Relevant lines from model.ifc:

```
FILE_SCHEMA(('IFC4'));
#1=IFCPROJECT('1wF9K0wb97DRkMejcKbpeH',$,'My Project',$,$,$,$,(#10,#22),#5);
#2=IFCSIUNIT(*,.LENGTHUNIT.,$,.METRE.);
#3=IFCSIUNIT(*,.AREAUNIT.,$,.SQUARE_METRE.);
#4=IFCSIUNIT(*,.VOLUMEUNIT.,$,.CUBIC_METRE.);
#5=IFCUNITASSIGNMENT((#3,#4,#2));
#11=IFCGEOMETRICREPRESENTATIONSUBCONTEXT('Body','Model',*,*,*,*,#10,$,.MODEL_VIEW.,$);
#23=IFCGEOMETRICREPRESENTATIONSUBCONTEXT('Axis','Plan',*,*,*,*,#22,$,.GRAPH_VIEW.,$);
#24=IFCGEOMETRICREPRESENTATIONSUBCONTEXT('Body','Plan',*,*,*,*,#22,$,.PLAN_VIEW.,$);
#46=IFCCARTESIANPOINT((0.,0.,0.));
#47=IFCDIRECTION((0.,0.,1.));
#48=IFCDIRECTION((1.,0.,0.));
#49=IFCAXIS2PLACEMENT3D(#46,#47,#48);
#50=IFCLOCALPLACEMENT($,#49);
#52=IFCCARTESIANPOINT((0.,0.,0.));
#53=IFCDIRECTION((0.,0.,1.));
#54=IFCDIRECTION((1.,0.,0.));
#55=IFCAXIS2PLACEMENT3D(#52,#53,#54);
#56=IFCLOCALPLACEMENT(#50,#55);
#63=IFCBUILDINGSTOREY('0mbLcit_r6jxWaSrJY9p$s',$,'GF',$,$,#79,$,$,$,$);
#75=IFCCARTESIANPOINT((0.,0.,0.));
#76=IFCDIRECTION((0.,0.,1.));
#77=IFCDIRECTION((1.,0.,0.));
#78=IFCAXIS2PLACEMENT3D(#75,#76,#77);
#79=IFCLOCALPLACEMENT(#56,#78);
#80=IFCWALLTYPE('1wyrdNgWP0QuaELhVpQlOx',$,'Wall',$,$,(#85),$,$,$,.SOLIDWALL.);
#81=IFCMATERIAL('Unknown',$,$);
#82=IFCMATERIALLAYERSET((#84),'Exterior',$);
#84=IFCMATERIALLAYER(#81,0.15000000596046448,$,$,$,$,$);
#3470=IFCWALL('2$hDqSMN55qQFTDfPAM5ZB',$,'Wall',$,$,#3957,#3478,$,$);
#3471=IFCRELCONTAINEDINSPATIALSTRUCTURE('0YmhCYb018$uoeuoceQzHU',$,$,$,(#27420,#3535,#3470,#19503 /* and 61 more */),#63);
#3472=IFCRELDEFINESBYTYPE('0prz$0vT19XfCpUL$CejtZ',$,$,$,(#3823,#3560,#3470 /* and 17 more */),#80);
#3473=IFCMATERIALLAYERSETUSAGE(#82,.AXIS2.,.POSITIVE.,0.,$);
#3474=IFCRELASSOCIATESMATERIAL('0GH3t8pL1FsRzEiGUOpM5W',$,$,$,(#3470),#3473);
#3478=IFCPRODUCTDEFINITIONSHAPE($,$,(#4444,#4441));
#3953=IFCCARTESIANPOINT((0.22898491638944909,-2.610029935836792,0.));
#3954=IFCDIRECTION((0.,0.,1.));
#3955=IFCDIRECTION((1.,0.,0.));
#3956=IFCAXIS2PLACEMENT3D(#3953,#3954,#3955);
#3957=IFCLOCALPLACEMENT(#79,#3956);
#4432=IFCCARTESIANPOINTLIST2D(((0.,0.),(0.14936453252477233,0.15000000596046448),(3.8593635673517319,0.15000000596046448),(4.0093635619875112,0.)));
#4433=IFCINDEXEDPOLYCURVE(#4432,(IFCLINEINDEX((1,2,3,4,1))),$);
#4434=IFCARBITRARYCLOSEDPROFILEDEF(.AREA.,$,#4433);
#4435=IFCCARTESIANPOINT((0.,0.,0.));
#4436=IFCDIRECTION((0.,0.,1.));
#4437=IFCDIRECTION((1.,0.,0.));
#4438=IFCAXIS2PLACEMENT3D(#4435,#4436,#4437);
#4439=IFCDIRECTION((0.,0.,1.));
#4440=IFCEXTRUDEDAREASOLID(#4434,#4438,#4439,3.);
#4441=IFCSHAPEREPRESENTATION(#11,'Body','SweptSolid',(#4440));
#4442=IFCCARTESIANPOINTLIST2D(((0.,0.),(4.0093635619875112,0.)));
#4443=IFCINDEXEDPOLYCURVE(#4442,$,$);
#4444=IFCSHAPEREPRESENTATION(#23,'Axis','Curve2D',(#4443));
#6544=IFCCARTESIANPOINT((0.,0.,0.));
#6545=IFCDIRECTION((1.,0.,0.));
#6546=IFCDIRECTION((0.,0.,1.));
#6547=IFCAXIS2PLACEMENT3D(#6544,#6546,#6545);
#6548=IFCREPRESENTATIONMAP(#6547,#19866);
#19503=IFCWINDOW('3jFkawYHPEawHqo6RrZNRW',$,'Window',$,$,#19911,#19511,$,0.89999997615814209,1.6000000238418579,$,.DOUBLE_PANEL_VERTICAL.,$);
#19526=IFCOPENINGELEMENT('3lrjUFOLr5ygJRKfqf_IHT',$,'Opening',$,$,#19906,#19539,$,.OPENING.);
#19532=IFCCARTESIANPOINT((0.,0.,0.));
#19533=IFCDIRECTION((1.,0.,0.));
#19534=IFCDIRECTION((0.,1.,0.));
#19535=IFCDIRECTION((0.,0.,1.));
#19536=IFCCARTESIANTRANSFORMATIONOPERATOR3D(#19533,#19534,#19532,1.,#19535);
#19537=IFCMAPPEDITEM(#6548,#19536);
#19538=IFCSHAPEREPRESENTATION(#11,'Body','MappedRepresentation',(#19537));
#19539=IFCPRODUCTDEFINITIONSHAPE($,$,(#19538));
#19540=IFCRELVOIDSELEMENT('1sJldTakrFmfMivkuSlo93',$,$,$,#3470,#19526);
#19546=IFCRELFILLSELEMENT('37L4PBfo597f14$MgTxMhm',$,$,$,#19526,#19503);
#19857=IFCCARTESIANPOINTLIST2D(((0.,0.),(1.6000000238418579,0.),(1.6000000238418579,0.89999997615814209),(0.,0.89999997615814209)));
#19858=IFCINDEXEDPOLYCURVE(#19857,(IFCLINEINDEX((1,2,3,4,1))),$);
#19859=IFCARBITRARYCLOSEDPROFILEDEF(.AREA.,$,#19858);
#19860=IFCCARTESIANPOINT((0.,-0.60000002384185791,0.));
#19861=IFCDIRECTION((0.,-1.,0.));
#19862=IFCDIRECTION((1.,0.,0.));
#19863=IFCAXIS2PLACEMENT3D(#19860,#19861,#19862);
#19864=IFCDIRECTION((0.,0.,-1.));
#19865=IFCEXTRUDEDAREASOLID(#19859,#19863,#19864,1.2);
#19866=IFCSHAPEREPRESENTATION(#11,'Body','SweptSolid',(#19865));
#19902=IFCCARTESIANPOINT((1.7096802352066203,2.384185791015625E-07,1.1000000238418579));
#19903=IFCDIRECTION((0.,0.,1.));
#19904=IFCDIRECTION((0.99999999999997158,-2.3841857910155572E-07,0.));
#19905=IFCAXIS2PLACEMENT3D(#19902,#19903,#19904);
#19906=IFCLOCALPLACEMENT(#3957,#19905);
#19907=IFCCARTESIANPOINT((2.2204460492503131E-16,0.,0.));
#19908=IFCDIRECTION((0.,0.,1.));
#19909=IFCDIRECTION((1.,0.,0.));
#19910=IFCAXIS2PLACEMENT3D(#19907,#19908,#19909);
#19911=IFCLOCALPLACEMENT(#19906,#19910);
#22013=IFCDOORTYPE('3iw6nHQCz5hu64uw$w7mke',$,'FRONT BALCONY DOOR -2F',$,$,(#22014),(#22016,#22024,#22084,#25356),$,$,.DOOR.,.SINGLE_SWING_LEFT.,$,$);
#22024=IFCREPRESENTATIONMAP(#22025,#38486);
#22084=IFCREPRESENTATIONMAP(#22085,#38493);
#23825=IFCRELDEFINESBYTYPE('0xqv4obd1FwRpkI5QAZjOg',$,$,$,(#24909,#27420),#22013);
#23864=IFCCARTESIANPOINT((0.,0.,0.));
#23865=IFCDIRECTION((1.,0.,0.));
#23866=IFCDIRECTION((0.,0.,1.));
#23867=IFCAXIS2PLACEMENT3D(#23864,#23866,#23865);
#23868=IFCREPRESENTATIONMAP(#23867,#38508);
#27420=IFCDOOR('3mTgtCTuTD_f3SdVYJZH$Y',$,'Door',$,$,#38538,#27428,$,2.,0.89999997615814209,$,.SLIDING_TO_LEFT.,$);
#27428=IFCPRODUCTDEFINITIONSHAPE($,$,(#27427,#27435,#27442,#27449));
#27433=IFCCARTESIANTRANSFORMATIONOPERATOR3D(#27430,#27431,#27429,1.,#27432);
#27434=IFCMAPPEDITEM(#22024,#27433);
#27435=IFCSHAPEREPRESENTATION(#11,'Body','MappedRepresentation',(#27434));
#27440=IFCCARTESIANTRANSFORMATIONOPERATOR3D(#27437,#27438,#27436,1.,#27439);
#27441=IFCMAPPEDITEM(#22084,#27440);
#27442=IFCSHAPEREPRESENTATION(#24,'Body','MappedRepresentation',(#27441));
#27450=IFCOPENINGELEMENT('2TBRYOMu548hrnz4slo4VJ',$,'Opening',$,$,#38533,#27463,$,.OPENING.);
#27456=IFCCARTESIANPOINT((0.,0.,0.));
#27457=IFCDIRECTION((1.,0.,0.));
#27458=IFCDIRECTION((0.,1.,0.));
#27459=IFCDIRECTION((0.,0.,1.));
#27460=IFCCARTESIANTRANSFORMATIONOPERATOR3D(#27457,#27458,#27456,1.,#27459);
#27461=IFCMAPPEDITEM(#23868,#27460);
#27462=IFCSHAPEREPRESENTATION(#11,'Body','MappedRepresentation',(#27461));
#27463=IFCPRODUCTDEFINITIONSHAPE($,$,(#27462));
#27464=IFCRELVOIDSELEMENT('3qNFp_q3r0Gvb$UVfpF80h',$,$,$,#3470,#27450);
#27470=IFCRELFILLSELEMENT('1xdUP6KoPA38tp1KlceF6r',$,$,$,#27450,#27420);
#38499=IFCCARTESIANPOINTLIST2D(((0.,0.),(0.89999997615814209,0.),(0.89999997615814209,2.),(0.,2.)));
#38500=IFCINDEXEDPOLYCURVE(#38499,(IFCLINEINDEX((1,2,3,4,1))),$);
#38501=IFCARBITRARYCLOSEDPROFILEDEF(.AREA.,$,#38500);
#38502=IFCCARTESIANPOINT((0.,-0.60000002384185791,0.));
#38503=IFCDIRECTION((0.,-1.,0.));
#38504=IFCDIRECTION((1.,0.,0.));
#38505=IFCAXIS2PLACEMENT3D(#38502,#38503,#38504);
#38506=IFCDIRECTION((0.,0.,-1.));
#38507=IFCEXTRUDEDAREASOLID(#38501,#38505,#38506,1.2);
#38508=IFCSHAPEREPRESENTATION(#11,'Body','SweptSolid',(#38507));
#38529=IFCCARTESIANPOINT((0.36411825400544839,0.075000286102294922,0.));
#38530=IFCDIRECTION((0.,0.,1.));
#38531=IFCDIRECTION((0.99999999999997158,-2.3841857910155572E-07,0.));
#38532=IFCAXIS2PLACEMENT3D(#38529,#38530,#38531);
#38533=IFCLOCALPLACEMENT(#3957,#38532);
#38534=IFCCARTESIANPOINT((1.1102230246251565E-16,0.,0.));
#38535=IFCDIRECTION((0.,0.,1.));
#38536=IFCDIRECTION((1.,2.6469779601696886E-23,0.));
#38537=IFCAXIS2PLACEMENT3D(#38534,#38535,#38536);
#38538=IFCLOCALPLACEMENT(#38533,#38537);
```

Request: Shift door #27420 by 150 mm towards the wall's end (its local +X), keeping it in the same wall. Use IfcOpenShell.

```python
import ifcopenshell
import ifcopenshell.api.geometry
import ifcopenshell.util.placement
import ifcopenshell.util.unit

model = ifcopenshell.open("model.ifc")
unit_scale = ifcopenshell.util.unit.calculate_unit_scale(model)

door = model.by_guid("3mTgtCTuTD_f3SdVYJZH$Y")
opening = door.FillsVoids[0].RelatingOpeningElement
wall = opening.VoidsElements[0].RelatingBuildingElement

wall_matrix = ifcopenshell.util.placement.get_local_placement(wall.ObjectPlacement)
shift = wall_matrix[:3, 0] * 0.15 / unit_scale
before = ifcopenshell.util.placement.get_local_placement(door.ObjectPlacement)[:3, 3].copy()

# The door is placed relative to its opening, so it follows when the opening moves.
matrix = ifcopenshell.util.placement.get_local_placement(opening.ObjectPlacement)
matrix[:3, 3] += shift
ifcopenshell.api.geometry.edit_object_placement(
    model, product=opening, matrix=matrix, is_si=False, should_transform_children=True
)

after = ifcopenshell.util.placement.get_local_placement(door.ObjectPlacement)[:3, 3]
print("door moved by", (after - before).round(3) + 0.0)

model.write("model_rev.ifc")
```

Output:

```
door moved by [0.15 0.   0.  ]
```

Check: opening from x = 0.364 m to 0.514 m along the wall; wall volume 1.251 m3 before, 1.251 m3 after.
